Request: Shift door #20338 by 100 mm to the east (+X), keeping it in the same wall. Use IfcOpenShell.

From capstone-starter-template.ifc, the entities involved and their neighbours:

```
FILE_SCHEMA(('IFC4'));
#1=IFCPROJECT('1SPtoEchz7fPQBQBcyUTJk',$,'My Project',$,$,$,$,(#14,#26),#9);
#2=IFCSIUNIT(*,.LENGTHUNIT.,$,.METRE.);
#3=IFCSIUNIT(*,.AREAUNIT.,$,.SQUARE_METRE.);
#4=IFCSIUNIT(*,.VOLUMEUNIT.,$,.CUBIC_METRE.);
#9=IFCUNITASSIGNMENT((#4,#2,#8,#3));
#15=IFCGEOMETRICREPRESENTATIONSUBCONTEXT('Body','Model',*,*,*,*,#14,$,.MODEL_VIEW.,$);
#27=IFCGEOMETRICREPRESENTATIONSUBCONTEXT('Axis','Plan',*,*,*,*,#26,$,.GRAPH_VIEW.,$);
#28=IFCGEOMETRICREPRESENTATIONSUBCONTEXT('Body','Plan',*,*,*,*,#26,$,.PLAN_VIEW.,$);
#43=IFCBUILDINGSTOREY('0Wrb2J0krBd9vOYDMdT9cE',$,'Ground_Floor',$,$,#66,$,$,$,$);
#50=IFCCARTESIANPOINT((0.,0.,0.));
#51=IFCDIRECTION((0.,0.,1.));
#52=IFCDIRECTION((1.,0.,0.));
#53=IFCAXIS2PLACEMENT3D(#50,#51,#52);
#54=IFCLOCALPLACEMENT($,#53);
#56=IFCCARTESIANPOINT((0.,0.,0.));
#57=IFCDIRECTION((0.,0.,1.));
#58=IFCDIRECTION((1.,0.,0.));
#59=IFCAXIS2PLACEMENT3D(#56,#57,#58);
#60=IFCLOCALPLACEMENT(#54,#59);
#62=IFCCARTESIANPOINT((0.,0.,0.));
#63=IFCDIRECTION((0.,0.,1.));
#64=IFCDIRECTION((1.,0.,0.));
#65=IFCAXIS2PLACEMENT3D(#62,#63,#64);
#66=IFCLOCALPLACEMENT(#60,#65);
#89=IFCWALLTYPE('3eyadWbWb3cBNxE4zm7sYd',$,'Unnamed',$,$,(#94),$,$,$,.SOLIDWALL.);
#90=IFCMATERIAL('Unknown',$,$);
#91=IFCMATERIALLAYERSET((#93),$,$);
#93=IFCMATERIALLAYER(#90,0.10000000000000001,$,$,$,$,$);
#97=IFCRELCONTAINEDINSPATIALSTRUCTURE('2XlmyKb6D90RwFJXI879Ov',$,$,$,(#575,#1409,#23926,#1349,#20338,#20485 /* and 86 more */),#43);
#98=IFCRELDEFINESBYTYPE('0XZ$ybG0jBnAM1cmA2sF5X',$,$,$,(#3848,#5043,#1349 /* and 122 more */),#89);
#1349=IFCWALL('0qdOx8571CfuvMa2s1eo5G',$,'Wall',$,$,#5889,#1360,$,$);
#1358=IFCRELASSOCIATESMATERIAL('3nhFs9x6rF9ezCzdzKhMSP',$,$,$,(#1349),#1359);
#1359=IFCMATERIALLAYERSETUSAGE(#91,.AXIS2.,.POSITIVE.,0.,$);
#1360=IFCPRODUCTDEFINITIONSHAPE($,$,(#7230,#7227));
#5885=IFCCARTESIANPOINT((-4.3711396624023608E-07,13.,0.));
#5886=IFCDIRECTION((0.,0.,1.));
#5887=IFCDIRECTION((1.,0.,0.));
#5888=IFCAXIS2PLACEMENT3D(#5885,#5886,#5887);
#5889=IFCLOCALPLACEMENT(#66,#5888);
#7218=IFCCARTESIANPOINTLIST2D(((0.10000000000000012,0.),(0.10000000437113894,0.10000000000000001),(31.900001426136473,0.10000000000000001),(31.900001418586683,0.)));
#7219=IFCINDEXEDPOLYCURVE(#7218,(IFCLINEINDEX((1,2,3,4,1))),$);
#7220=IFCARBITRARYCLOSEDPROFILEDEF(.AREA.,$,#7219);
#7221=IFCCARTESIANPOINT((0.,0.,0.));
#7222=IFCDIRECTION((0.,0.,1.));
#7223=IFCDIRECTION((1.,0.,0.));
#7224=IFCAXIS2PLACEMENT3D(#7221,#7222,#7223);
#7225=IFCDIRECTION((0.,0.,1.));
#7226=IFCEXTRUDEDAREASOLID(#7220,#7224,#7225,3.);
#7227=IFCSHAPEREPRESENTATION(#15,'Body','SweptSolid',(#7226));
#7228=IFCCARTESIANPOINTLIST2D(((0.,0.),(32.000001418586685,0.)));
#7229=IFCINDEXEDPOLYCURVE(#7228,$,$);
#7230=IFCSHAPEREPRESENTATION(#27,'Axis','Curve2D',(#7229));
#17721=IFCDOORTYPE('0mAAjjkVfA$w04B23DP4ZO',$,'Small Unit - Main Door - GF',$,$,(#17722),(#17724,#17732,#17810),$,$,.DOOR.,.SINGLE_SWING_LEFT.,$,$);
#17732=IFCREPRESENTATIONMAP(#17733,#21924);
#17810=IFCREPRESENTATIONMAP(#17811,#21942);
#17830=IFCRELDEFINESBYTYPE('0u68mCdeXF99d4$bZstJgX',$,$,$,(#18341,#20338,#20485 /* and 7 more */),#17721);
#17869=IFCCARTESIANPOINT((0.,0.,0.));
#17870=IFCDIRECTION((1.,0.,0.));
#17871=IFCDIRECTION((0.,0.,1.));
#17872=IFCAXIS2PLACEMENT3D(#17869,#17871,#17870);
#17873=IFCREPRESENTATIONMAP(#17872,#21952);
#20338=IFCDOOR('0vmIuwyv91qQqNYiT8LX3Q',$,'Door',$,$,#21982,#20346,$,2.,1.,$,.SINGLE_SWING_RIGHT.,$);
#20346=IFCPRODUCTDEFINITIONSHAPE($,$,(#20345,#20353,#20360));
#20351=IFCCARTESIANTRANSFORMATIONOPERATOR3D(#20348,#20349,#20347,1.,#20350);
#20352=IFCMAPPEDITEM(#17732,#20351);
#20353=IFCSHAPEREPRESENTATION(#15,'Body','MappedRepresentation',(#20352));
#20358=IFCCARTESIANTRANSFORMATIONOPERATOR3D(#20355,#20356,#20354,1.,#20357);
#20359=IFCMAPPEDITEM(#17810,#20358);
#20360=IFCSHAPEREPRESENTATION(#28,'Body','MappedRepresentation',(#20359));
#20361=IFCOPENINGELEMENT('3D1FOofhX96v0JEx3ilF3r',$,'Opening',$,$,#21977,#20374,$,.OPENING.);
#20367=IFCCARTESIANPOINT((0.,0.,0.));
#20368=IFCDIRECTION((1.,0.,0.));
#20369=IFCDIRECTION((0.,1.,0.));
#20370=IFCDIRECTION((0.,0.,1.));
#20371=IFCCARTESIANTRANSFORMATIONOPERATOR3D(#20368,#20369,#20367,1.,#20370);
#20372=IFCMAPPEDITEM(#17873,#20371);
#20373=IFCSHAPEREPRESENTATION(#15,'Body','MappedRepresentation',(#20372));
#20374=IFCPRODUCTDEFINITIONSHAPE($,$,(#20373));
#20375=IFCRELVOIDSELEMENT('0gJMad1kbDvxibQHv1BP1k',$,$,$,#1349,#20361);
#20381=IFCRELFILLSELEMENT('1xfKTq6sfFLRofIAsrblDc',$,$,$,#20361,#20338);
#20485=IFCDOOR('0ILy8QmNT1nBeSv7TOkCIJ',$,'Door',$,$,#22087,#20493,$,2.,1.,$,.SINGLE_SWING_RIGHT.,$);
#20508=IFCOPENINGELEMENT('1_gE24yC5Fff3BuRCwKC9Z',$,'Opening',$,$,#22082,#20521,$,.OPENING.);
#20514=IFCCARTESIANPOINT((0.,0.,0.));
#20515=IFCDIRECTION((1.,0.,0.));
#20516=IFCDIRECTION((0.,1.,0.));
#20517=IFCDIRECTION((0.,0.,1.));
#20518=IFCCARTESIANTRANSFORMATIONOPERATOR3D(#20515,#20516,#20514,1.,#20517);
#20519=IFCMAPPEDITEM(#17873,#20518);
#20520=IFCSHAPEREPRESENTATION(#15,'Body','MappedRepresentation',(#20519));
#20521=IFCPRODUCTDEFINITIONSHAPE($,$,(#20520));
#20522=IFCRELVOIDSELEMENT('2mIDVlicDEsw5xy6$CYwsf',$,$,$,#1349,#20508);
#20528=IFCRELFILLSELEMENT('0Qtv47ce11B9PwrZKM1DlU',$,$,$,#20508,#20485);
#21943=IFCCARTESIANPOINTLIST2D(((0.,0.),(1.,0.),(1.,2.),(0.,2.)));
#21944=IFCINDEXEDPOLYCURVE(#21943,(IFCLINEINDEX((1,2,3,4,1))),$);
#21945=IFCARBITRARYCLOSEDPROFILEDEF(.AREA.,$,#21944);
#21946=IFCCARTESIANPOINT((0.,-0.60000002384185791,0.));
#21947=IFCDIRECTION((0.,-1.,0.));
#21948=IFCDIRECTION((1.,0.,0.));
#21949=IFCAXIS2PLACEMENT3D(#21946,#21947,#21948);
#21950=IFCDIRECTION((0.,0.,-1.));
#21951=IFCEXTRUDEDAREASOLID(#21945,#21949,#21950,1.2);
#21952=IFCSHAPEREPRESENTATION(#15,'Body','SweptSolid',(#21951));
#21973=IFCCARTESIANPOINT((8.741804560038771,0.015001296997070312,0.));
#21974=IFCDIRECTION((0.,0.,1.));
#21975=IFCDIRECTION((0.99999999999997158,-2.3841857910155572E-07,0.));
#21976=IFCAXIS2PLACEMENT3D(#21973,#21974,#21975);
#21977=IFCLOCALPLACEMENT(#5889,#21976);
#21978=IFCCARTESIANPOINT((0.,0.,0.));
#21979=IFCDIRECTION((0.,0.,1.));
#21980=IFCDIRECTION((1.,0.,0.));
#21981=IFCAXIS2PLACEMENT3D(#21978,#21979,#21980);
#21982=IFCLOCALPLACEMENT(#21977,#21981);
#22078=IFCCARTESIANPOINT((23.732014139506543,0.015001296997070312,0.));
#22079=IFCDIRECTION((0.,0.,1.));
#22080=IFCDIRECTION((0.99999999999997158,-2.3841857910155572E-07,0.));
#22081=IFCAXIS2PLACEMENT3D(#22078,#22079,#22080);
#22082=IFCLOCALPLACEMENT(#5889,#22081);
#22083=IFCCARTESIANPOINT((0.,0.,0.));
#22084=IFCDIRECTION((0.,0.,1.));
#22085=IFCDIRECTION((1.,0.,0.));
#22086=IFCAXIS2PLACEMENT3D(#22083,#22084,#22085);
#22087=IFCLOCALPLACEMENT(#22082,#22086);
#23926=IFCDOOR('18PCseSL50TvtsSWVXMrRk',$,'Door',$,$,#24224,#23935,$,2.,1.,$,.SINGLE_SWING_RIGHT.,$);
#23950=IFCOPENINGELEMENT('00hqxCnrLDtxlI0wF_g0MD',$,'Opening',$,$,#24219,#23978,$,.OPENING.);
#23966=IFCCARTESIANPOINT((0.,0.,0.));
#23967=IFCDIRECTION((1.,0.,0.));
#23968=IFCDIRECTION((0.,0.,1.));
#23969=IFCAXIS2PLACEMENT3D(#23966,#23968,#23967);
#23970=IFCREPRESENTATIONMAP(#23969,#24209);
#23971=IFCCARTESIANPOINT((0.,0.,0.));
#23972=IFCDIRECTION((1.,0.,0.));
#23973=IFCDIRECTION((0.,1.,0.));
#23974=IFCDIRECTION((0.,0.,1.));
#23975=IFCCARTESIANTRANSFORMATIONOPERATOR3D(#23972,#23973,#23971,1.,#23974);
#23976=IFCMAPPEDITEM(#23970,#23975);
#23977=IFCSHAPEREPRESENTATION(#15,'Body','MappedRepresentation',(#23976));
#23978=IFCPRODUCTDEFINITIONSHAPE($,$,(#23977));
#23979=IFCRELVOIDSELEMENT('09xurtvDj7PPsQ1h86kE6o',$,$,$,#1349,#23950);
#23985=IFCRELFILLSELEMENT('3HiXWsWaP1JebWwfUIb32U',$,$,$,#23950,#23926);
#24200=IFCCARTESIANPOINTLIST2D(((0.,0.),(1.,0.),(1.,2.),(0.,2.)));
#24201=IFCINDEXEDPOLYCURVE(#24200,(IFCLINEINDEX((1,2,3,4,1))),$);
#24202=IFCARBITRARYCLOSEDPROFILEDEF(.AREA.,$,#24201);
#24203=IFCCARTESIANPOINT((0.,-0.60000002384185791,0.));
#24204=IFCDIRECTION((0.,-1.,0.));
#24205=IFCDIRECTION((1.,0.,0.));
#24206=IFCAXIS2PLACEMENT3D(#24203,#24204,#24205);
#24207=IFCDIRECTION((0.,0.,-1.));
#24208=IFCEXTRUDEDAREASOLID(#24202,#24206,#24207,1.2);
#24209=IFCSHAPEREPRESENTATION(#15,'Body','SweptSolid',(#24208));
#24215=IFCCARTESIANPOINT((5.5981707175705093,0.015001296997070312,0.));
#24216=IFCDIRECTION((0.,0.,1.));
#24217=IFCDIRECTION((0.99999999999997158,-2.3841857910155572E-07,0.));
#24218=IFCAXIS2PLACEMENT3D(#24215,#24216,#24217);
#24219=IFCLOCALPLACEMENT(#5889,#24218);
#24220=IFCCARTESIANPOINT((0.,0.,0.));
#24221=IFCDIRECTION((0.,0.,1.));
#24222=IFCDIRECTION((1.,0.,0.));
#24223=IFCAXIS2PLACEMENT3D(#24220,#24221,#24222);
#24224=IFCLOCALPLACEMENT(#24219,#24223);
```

```python
import ifcopenshell
import ifcopenshell.api.geometry
import ifcopenshell.util.placement
import ifcopenshell.util.unit

model = ifcopenshell.open("capstone-starter-template.ifc")
unit_scale = ifcopenshell.util.unit.calculate_unit_scale(model)

door = model.by_guid("0vmIuwyv91qQqNYiT8LX3Q")
opening = door.FillsVoids[0].RelatingOpeningElement
wall = opening.VoidsElements[0].RelatingBuildingElement

wall_matrix = ifcopenshell.util.placement.get_local_placement(wall.ObjectPlacement)
shift = wall_matrix[:3, 0] * 0.1 / unit_scale
before = ifcopenshell.util.placement.get_local_placement(door.ObjectPlacement)[:3, 3].copy()

# The door is placed relative to its opening, so it follows when the opening moves.
matrix = ifcopenshell.util.placement.get_local_placement(opening.ObjectPlacement)
matrix[:3, 3] += shift
ifcopenshell.api.geometry.edit_object_placement(
    model, product=opening, matrix=matrix, is_si=False, should_transform_children=True
)

after = ifcopenshell.util.placement.get_local_placement(door.ObjectPlacement)[:3, 3]
print("door moved by", (after - before).round(3) + 0.0)

model.write("capstone-starter-template_edited.ifc")
```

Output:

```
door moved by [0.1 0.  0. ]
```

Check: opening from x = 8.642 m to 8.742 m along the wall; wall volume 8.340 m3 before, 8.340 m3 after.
